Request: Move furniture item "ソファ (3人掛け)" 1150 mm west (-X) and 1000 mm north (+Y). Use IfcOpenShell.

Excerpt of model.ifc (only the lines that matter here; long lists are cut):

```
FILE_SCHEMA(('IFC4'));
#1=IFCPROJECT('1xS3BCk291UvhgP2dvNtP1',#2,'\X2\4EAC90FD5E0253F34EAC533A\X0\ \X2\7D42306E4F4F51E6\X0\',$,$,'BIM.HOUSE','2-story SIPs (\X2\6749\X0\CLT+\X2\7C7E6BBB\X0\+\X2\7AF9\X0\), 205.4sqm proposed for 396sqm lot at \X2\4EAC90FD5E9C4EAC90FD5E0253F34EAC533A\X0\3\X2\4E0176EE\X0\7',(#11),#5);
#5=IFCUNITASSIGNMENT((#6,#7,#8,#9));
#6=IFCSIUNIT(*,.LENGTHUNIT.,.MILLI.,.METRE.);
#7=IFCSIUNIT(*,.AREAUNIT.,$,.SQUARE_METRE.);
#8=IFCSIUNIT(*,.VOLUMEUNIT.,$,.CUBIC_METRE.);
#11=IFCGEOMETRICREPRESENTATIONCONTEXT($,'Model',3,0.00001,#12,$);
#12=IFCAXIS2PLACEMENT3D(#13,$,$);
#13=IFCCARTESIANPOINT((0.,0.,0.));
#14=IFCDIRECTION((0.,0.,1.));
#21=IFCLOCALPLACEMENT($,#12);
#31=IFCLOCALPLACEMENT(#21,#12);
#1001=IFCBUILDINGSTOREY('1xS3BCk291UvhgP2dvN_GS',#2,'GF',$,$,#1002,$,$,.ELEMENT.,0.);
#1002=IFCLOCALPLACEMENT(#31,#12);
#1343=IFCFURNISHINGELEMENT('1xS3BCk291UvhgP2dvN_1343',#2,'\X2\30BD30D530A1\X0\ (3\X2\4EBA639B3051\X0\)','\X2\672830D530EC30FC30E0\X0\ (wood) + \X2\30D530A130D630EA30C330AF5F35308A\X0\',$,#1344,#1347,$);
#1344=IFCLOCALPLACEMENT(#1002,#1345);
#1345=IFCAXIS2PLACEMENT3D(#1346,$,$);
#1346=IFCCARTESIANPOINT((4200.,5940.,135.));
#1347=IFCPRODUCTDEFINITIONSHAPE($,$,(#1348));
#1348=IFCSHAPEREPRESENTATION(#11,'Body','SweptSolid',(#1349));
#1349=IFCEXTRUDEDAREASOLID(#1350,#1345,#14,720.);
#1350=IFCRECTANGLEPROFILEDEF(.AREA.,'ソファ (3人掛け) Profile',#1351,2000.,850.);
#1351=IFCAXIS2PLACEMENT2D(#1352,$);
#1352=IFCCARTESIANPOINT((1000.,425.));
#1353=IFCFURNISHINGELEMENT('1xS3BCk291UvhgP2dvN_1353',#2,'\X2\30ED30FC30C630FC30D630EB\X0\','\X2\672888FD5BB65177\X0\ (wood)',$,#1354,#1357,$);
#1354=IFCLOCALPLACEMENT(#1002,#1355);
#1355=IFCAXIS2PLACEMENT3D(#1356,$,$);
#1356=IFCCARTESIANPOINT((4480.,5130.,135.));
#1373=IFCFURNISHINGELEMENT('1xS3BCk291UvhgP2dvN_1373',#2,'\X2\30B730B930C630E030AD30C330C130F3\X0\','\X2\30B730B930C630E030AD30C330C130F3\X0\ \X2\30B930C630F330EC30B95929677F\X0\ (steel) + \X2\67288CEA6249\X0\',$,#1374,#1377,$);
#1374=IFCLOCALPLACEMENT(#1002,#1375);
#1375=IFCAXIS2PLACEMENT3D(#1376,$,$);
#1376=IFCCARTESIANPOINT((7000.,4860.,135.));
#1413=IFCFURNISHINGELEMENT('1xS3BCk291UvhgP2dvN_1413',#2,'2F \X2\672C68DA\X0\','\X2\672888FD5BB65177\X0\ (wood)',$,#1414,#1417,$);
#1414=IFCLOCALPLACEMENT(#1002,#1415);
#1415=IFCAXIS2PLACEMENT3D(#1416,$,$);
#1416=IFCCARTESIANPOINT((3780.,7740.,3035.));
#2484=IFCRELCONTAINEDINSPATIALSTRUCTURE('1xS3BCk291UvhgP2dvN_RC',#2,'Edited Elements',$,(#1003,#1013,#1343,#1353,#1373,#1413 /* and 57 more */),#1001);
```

```python
import ifcopenshell
import ifcopenshell.api.geometry
import ifcopenshell.util.placement
import ifcopenshell.util.unit

model = ifcopenshell.open("model.ifc")
unit_scale = ifcopenshell.util.unit.calculate_unit_scale(model)

item = model.by_guid("1xS3BCk291UvhgP2dvN_1343")
matrix = ifcopenshell.util.placement.get_local_placement(item.ObjectPlacement)
matrix[0, 3] -= 1.15 / unit_scale
matrix[1, 3] += 1 / unit_scale
ifcopenshell.api.geometry.edit_object_placement(model, product=item, matrix=matrix, is_si=False)

print(ifcopenshell.util.placement.get_local_placement(item.ObjectPlacement).round(3) + 0.0)

model.write("model_v2.ifc")
```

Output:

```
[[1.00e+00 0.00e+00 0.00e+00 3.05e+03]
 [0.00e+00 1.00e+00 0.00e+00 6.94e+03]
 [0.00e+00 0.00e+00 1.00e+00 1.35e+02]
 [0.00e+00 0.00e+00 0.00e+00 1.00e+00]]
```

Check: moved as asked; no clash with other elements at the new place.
